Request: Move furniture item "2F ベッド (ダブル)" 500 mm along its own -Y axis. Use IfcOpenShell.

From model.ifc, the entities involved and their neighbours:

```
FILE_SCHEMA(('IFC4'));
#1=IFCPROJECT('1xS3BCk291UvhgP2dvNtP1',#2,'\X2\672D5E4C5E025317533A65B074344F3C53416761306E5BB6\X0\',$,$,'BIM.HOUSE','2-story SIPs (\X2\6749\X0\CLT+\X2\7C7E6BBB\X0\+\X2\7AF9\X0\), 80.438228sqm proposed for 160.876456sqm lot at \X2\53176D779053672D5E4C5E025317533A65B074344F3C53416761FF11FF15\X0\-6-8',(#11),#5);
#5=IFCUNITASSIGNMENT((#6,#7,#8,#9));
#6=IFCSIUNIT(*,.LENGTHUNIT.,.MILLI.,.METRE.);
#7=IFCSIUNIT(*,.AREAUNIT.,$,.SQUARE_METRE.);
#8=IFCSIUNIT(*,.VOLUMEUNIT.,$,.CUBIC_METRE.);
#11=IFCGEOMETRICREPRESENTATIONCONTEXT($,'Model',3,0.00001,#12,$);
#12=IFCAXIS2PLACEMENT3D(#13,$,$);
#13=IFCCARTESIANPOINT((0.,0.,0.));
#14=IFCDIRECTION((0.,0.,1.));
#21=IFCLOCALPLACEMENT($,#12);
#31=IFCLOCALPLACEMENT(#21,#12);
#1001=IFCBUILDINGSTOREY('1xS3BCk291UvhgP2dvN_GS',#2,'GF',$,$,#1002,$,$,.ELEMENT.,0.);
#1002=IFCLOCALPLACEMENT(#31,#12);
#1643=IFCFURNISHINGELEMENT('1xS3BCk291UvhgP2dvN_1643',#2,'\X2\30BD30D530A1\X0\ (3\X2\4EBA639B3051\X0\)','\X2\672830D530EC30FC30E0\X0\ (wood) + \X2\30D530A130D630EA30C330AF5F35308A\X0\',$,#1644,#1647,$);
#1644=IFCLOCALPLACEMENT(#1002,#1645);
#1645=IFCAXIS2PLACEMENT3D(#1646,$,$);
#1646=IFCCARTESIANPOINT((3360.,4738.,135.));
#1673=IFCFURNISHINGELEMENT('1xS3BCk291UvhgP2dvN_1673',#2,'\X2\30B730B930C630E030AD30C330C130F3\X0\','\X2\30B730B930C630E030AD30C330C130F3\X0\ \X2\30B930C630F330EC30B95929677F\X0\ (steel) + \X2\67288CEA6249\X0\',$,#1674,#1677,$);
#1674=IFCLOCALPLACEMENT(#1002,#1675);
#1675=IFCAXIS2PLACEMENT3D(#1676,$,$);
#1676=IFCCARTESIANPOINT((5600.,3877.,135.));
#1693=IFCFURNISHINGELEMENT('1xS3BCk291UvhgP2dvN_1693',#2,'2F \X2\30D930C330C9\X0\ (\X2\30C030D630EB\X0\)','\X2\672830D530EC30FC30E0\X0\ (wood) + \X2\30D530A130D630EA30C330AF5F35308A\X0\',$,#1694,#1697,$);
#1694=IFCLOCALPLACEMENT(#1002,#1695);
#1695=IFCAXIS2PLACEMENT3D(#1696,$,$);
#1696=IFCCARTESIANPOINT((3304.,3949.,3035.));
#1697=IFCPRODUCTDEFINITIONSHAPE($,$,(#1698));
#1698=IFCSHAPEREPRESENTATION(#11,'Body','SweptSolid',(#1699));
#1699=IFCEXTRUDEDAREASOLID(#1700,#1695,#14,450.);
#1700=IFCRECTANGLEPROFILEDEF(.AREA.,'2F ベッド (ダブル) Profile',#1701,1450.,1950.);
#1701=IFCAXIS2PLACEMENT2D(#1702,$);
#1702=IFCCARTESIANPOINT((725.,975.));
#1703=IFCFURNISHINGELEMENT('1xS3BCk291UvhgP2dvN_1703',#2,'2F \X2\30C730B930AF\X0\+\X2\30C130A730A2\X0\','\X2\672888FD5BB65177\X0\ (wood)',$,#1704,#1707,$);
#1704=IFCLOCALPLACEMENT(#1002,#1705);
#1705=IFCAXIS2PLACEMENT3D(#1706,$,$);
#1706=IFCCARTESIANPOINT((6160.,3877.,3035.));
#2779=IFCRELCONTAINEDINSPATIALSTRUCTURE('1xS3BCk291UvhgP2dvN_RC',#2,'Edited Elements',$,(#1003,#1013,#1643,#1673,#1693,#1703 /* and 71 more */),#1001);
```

```python
import ifcopenshell
import ifcopenshell.api.geometry
import ifcopenshell.util.placement
import ifcopenshell.util.unit

model = ifcopenshell.open("model.ifc")
unit_scale = ifcopenshell.util.unit.calculate_unit_scale(model)

item = model.by_guid("1xS3BCk291UvhgP2dvN_1693")
matrix = ifcopenshell.util.placement.get_local_placement(item.ObjectPlacement)
matrix[:3, 3] -= matrix[:3, 1] * 0.5 / unit_scale
ifcopenshell.api.geometry.edit_object_placement(model, product=item, matrix=matrix, is_si=False)

print(ifcopenshell.util.placement.get_local_placement(item.ObjectPlacement).round(3) + 0.0)

model.write("model_edited.ifc")
```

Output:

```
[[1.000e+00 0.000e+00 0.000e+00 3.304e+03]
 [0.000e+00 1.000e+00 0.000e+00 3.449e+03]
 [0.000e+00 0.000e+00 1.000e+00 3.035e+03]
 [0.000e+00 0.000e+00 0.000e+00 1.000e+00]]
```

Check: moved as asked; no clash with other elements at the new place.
